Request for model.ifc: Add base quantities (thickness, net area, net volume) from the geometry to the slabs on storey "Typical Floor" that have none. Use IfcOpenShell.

First a look at what the model holds.

```python
import ifcopenshell
import ifcopenshell.util.element
import ifcopenshell.util.unit

model = ifcopenshell.open("model.ifc")
print(model.schema)
for unit_type in ("LENGTHUNIT", "AREAUNIT", "VOLUMEUNIT"):
    print(unit_type, ifcopenshell.util.unit.calculate_unit_scale(model, unit_type))
storey = next(s for s in model.by_type("IfcBuildingStorey") if s.Name == "Typical Floor")
slabs = [e for e in ifcopenshell.util.element.get_decomposition(storey) if e.is_a("IfcSlab")]
for e in sorted(slabs, key=lambda e: e.id()):
    print(e.id(), e.is_a(), e.Name, list(ifcopenshell.util.element.get_psets(e, qtos_only=True)), sep=" | ")
```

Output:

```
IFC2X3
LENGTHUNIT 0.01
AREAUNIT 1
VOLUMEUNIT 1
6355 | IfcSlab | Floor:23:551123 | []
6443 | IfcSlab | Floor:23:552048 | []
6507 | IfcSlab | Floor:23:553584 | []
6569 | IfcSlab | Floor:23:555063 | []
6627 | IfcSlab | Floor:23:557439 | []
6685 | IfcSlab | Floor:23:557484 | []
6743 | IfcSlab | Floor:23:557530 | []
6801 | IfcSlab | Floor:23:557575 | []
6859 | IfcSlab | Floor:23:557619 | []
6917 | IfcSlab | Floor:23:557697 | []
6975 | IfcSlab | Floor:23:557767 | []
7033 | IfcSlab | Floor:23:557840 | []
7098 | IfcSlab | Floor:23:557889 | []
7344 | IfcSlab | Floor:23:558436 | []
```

```python
import ifcopenshell
import ifcopenshell.api.pset
import ifcopenshell.geom
import ifcopenshell.util.element
import ifcopenshell.util.shape
import ifcopenshell.util.unit

model = ifcopenshell.open("model.ifc")
unit_scale = ifcopenshell.util.unit.calculate_unit_scale(model)
area_scale = ifcopenshell.util.unit.calculate_unit_scale(model, "AREAUNIT")
volume_scale = ifcopenshell.util.unit.calculate_unit_scale(model, "VOLUMEUNIT")
settings = ifcopenshell.geom.settings()

storey = next(s for s in model.by_type("IfcBuildingStorey") if s.Name == "Typical Floor")
slabs = [e for e in ifcopenshell.util.element.get_decomposition(storey) if e.is_a("IfcSlab")]

for e in sorted(slabs, key=lambda e: e.id()):
    if ifcopenshell.util.element.get_psets(e, qtos_only=True, should_inherit=False):
        continue
    # Geometry comes back in metres, in the element's own axes.
    shape = ifcopenshell.geom.create_shape(settings, e)
    values = {
        "Width": ifcopenshell.util.shape.get_z(shape.geometry) / unit_scale,
        "NetArea": ifcopenshell.util.shape.get_footprint_area(shape.geometry) / area_scale,
        "NetVolume": ifcopenshell.util.shape.get_volume(shape.geometry) / volume_scale,
    }
    qto = ifcopenshell.api.pset.add_qto(model, product=e, name="BaseQuantities")
    ifcopenshell.api.pset.edit_qto(model, qto=qto, properties=values)
    print(e.id(), {k: round(v, 3) for k, v in values.items()})

model.write("model_rev.ifc")
```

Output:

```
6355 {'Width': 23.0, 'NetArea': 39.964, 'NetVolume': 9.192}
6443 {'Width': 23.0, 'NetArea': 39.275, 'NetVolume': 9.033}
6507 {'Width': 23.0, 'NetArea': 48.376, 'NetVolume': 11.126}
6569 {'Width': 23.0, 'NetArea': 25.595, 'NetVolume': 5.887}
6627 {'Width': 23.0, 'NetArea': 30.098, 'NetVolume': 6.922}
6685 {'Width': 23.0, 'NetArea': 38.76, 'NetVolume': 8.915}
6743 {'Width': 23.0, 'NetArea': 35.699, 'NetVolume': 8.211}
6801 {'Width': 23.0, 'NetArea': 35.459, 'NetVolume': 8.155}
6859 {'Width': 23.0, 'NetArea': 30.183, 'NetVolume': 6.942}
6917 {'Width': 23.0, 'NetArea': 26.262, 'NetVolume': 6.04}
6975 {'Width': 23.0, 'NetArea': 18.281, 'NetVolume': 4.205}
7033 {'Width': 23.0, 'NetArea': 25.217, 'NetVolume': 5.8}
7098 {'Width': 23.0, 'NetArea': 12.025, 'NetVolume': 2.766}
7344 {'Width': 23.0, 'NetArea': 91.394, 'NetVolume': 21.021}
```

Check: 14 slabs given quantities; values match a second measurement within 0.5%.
